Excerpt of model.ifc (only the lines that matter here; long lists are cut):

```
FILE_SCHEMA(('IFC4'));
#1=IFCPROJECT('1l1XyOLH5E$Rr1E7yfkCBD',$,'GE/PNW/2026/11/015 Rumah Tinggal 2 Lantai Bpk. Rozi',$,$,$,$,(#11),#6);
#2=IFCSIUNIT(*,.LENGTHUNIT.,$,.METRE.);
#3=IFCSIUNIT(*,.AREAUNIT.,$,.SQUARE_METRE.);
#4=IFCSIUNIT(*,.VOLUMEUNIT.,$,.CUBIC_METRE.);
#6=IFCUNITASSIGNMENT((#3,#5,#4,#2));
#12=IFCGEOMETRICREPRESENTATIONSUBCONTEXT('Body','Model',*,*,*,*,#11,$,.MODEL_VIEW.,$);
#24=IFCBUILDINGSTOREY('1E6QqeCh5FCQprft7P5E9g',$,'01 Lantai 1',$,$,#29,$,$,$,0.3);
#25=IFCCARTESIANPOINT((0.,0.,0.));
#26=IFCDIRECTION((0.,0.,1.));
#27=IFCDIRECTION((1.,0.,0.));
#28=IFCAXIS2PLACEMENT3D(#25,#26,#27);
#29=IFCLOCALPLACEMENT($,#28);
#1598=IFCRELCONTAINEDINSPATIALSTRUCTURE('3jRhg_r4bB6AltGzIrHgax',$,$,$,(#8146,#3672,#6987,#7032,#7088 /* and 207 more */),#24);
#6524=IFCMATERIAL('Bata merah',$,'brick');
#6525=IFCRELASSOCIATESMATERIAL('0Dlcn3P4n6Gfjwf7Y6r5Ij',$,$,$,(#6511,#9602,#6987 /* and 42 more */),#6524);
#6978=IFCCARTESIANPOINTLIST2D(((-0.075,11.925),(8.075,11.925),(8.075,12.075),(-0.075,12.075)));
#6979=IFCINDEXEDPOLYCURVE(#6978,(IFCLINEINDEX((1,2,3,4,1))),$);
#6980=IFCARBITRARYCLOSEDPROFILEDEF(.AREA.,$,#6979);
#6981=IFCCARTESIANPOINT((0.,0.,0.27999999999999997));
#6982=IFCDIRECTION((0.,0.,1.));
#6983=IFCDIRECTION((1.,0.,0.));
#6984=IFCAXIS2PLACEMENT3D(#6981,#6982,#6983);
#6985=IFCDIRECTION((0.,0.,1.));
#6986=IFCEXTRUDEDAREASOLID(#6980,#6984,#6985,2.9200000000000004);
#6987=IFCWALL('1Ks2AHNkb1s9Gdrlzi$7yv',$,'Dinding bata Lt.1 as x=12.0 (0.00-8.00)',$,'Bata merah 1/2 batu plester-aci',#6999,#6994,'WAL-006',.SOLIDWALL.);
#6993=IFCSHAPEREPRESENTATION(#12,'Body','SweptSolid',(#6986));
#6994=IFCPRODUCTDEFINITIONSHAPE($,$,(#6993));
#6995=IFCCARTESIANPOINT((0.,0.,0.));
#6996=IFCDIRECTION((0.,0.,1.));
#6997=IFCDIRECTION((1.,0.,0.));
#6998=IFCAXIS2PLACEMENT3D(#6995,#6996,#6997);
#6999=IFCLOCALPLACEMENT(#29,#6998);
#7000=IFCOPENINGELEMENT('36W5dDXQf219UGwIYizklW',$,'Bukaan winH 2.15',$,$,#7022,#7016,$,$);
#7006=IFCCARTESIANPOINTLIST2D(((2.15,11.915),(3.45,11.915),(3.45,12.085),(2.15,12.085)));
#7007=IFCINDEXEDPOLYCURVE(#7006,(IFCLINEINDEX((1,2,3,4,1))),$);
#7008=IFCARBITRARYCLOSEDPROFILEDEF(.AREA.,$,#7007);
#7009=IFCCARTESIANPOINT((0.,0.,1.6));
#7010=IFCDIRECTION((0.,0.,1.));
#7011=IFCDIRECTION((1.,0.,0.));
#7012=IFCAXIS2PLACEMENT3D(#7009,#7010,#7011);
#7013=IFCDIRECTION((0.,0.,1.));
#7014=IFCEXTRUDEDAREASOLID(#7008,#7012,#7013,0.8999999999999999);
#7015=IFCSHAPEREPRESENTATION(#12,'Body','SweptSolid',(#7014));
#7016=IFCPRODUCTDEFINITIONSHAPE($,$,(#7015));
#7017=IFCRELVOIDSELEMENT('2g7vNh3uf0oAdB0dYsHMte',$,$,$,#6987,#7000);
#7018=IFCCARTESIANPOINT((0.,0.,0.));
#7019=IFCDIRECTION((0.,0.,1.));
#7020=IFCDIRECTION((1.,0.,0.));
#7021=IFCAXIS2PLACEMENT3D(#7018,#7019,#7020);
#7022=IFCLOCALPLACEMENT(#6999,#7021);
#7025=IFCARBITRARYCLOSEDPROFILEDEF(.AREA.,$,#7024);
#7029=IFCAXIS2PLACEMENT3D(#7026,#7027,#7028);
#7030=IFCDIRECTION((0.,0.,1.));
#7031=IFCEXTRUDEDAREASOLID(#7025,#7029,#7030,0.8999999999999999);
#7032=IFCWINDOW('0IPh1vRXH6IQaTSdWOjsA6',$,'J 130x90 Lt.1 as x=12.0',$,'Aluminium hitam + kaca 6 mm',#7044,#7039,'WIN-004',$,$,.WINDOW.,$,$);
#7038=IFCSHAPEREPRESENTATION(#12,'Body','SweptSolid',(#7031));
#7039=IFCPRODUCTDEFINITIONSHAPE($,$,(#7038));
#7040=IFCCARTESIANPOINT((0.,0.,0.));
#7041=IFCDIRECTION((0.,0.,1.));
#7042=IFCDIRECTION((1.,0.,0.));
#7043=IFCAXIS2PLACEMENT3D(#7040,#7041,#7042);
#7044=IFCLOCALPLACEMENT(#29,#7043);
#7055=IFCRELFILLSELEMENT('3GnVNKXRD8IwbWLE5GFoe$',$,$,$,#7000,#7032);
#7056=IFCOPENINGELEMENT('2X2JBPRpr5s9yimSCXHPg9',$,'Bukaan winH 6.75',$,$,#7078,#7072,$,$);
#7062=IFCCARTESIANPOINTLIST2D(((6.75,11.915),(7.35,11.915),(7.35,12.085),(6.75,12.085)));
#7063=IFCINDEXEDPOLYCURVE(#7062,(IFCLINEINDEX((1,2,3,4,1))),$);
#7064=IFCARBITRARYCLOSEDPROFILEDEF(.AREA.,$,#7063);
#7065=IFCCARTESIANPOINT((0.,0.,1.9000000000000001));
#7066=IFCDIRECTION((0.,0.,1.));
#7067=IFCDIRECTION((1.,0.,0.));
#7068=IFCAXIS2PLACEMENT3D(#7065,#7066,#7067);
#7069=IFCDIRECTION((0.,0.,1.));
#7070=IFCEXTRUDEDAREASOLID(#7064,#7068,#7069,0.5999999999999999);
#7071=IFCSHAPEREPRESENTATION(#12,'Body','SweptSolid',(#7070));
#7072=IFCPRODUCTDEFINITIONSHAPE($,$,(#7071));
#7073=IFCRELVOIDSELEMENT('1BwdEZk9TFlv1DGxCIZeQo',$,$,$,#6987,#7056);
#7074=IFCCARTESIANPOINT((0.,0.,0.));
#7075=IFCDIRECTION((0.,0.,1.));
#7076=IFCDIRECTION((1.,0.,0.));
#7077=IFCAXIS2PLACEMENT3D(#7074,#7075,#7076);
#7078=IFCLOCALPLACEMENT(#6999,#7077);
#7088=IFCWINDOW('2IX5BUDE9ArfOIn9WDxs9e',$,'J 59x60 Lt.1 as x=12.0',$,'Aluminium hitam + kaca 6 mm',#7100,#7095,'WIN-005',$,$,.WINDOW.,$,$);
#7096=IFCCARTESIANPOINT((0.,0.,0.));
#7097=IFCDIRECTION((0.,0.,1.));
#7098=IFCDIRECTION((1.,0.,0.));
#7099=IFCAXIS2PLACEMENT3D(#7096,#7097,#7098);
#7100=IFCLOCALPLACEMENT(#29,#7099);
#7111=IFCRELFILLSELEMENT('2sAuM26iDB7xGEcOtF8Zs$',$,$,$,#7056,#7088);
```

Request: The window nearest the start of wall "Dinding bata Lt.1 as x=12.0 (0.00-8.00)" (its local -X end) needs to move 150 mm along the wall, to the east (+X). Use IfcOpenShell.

```python
import ifcopenshell
import ifcopenshell.api.geometry
import ifcopenshell.util.placement
import ifcopenshell.util.unit

model = ifcopenshell.open("model.ifc")
unit_scale = ifcopenshell.util.unit.calculate_unit_scale(model)

window = model.by_id(7032)
opening = window.FillsVoids[0].RelatingOpeningElement
wall = opening.VoidsElements[0].RelatingBuildingElement

wall_matrix = ifcopenshell.util.placement.get_local_placement(wall.ObjectPlacement)
shift = wall_matrix[:3, 0] * 0.15 / unit_scale
before = ifcopenshell.util.placement.get_local_placement(window.ObjectPlacement)[:3, 3].copy()

# The window is not placed relative to its opening, so move both.
for product in (opening, window):
    matrix = ifcopenshell.util.placement.get_local_placement(product.ObjectPlacement)
    matrix[:3, 3] += shift
    ifcopenshell.api.geometry.edit_object_placement(model, product=product, matrix=matrix, is_si=False)

after = ifcopenshell.util.placement.get_local_placement(window.ObjectPlacement)[:3, 3]
print("window moved by", (after - before).round(3) + 0.0)

model.write("model_updated.ifc")
```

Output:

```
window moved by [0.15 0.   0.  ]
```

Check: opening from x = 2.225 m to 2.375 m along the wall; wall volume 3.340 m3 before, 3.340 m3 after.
